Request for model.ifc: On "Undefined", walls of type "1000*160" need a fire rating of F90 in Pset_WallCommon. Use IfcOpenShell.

First a look at what the model holds.

```python
import ifcopenshell
import ifcopenshell.util.element

model = ifcopenshell.open("model.ifc")
print(model.schema)
storey = next(s for s in model.by_type("IfcBuildingStorey") if s.Name == "Undefined")
walls = [e for e in ifcopenshell.util.element.get_decomposition(storey) if e.is_a("IfcWall")]
seen = {}
for e in walls:
    element_type = ifcopenshell.util.element.get_type(e)
    key = (element_type.Name if element_type != e and element_type else None, ifcopenshell.util.element.get_pset(e, "Pset_WallCommon", "FireRating"))
    seen[key] = seen.get(key, 0) + 1
for (name, value), count in sorted(seen.items(), key=str):
    print(count, "x", name, "|", value)
```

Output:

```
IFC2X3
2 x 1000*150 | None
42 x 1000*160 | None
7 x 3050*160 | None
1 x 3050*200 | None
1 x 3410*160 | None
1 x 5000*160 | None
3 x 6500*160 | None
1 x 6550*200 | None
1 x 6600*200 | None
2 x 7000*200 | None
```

```python
import ifcopenshell
import ifcopenshell.api.pset
import ifcopenshell.util.element

model = ifcopenshell.open("model.ifc")

storey = next(s for s in model.by_type("IfcBuildingStorey") if s.Name == "Undefined")
walls = [e for e in ifcopenshell.util.element.get_decomposition(storey) if e.is_a("IfcWall")]

count = 0
for e in walls:
    element_type = ifcopenshell.util.element.get_type(e)
    if element_type in (None, e) or element_type.Name != "1000*160":
        continue
    # add_pset returns the element's existing set when there is one.
    pset = ifcopenshell.api.pset.add_pset(model, product=e, name="Pset_WallCommon")
    ifcopenshell.api.pset.edit_pset(model, pset=pset, properties={"FireRating": "F90"})
    count += 1

print(count, "walls updated")

model.write("model-out.ifc")
```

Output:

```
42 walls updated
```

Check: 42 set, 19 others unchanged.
